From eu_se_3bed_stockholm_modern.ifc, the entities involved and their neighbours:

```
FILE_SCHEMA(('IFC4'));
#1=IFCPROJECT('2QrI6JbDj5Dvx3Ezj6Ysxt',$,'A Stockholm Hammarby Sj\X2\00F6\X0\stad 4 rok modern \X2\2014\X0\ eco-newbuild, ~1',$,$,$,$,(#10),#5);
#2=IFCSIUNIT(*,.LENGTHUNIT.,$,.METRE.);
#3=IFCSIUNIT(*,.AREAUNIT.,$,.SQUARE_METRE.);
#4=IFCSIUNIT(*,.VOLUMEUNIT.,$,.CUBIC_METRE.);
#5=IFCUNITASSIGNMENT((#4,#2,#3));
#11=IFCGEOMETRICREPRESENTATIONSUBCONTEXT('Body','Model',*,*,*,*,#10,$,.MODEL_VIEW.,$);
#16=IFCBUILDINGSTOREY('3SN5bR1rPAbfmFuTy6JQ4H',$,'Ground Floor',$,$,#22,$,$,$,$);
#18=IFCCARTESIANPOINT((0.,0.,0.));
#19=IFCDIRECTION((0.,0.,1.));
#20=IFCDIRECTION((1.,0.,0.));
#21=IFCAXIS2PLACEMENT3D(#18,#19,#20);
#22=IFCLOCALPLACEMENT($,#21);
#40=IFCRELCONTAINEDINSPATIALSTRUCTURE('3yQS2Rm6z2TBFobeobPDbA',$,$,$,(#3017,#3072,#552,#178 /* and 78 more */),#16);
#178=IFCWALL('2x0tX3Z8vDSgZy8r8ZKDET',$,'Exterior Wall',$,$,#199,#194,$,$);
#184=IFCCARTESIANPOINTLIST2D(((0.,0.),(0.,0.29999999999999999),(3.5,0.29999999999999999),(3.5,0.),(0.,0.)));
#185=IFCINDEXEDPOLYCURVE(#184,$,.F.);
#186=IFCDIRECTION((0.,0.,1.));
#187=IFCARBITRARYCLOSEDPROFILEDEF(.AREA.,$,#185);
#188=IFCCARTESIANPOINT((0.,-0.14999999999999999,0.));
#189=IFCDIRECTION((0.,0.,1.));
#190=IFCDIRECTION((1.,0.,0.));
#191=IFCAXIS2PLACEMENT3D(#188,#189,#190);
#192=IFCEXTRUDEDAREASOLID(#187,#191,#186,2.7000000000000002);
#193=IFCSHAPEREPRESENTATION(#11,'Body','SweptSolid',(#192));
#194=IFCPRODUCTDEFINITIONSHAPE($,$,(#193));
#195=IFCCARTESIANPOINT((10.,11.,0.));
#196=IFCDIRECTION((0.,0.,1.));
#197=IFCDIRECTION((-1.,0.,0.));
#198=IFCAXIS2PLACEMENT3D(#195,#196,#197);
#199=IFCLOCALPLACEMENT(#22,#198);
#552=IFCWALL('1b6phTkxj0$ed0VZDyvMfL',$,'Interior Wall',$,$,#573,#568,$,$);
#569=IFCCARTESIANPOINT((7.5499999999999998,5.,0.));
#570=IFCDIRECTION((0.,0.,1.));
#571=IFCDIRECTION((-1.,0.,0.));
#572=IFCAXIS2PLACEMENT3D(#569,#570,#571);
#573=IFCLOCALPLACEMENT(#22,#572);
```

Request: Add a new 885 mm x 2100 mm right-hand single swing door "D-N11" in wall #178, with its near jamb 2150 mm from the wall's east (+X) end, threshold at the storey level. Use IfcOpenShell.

```python
import numpy as np
import ifcopenshell
import ifcopenshell.api.feature
import ifcopenshell.api.geometry
import ifcopenshell.api.root
import ifcopenshell.api.spatial
import ifcopenshell.geom
import ifcopenshell.util.element
import ifcopenshell.util.placement
import ifcopenshell.util.representation
import ifcopenshell.util.shape
import ifcopenshell.util.unit

model = ifcopenshell.open("eu_se_3bed_stockholm_modern.ifc")
unit_scale = ifcopenshell.util.unit.calculate_unit_scale(model)
settings = ifcopenshell.geom.settings()


def volume(element):
    """Net volume in cubic metres, openings subtracted."""
    shape = ifcopenshell.geom.create_shape(settings, element)
    return ifcopenshell.util.shape.get_volume(shape.geometry)


wall = model.by_guid("2x0tX3Z8vDSgZy8r8ZKDET")
storey = ifcopenshell.util.element.get_container(wall, ifc_class="IfcBuildingStorey")
context = ifcopenshell.util.representation.get_context(model, "Model", "Body", "MODEL_VIEW")
before = volume(wall)

width, height, from_end, sill = 0.885, 2.1, 2.15, 0.0  # metres

# The wall runs along its own X axis, and the end named is its -X end.
wall_shape = ifcopenshell.geom.create_shape(settings, wall)
x, y, z = ifcopenshell.util.shape.get_vertices(wall_shape.geometry).T
start = x.min() + from_end
face, thickness = float(y.min()), float(y.max() - y.min())
wall_matrix = ifcopenshell.util.placement.get_local_placement(wall.ObjectPlacement)
level = ifcopenshell.util.placement.get_local_placement(storey.ObjectPlacement)[2, 3]


def in_wall(x, y):
    """Placement at x, y metres in the wall's axes, at sill height."""
    matrix = wall_matrix.copy()
    matrix[:, 3] = wall_matrix @ np.array([x / unit_scale, y / unit_scale, 0.0, 1.0])
    matrix[2, 3] = level + sill / unit_scale
    return matrix


# Opening: a box that overshoots both wall faces by 50 mm.
opening = ifcopenshell.api.root.create_entity(model, ifc_class="IfcOpeningElement", predefined_type="OPENING")
box = ifcopenshell.api.geometry.add_wall_representation(
    model, context=context, length=width, height=height, thickness=thickness + 0.1
)
ifcopenshell.api.geometry.assign_representation(model, product=opening, representation=box)
ifcopenshell.api.geometry.edit_object_placement(model, product=opening, matrix=in_wall(start, face - 0.05), is_si=False)
ifcopenshell.api.feature.add_feature(model, feature=opening, element=wall)

door = ifcopenshell.api.root.create_entity(model, ifc_class="IfcDoor", name="D-N11", predefined_type="DOOR")
door.OverallWidth, door.OverallHeight = width / unit_scale, height / unit_scale
door.OperationType = "SINGLE_SWING_RIGHT"
body = ifcopenshell.api.geometry.add_door_representation(
    model,
    context=context,
    overall_width=door.OverallWidth,
    overall_height=door.OverallHeight,
    operation_type="SINGLE_SWING_RIGHT",
    lining_properties={"LiningDepth": thickness / unit_scale, "ThresholdDepth": thickness / unit_scale},
)
ifcopenshell.api.geometry.assign_representation(model, product=door, representation=body)
ifcopenshell.api.spatial.assign_container(model, products=[door], relating_structure=storey)
ifcopenshell.api.feature.add_filling(model, opening=opening, element=door)

# The lining spans the wall, so the door starts at the wall face.
ifcopenshell.api.geometry.edit_object_placement(model, product=door, matrix=in_wall(start, face), is_si=False)

after = volume(wall)

print(f"wall volume {before:.3f} -> {after:.3f} m3")

model.write("eu_se_3bed_stockholm_modern_rev.ifc")
```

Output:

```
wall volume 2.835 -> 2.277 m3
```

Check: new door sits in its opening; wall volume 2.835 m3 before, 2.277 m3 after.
